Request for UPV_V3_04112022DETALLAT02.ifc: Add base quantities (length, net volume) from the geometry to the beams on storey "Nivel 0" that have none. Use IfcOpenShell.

First a look at what the model holds.

```python
import ifcopenshell
import ifcopenshell.util.element
import ifcopenshell.util.unit

model = ifcopenshell.open("UPV_V3_04112022DETALLAT02.ifc")
print(model.schema)
for unit_type in ("LENGTHUNIT", "AREAUNIT", "VOLUMEUNIT"):
    print(unit_type, ifcopenshell.util.unit.calculate_unit_scale(model, unit_type))
storey = next(s for s in model.by_type("IfcBuildingStorey") if s.Name == "Nivel 0")
beams = [e for e in ifcopenshell.util.element.get_decomposition(storey) if e.is_a("IfcBeam")]
for e in sorted(beams, key=lambda e: e.id()):
    print(e.id(), e.is_a(), e.Name, list(ifcopenshell.util.element.get_psets(e, qtos_only=True)), sep=" | ")
```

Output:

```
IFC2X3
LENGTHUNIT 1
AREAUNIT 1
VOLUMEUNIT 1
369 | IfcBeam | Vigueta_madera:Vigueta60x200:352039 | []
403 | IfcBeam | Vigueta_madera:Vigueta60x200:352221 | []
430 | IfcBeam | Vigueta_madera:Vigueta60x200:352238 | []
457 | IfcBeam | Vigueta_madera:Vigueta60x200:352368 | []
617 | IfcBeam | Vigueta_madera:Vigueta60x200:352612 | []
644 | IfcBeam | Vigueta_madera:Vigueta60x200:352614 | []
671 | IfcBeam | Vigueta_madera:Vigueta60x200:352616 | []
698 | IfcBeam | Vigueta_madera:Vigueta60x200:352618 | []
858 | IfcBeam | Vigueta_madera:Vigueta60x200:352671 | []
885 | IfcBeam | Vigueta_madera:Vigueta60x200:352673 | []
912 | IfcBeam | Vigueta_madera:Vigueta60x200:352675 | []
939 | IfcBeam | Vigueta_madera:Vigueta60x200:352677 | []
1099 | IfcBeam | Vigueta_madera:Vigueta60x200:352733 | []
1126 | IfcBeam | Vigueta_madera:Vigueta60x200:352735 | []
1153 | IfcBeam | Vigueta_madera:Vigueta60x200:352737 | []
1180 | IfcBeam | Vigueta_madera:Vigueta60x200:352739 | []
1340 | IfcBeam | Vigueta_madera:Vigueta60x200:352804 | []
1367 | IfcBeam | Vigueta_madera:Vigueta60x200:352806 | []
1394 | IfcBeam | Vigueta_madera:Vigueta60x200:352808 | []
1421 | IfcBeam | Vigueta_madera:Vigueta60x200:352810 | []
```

```python
import ifcopenshell
import ifcopenshell.api.pset
import ifcopenshell.geom
import ifcopenshell.util.element
import ifcopenshell.util.shape
import ifcopenshell.util.unit

model = ifcopenshell.open("UPV_V3_04112022DETALLAT02.ifc")
unit_scale = ifcopenshell.util.unit.calculate_unit_scale(model)
volume_scale = ifcopenshell.util.unit.calculate_unit_scale(model, "VOLUMEUNIT")
settings = ifcopenshell.geom.settings()

storey = next(s for s in model.by_type("IfcBuildingStorey") if s.Name == "Nivel 0")
beams = [e for e in ifcopenshell.util.element.get_decomposition(storey) if e.is_a("IfcBeam")]

for e in sorted(beams, key=lambda e: e.id()):
    if ifcopenshell.util.element.get_psets(e, qtos_only=True, should_inherit=False):
        continue
    # Geometry comes back in metres, in the element's own axes.
    shape = ifcopenshell.geom.create_shape(settings, e)
    values = {
        "Length": ifcopenshell.util.shape.get_max_xyz(shape.geometry) / unit_scale,
        "NetVolume": ifcopenshell.util.shape.get_volume(shape.geometry) / volume_scale,
    }
    qto = ifcopenshell.api.pset.add_qto(model, product=e, name="BaseQuantities")
    ifcopenshell.api.pset.edit_qto(model, qto=qto, properties=values)
    print(e.id(), {k: round(v, 3) for k, v in values.items()})

model.write("UPV_V3_04112022DETALLAT02_v2.ifc")
```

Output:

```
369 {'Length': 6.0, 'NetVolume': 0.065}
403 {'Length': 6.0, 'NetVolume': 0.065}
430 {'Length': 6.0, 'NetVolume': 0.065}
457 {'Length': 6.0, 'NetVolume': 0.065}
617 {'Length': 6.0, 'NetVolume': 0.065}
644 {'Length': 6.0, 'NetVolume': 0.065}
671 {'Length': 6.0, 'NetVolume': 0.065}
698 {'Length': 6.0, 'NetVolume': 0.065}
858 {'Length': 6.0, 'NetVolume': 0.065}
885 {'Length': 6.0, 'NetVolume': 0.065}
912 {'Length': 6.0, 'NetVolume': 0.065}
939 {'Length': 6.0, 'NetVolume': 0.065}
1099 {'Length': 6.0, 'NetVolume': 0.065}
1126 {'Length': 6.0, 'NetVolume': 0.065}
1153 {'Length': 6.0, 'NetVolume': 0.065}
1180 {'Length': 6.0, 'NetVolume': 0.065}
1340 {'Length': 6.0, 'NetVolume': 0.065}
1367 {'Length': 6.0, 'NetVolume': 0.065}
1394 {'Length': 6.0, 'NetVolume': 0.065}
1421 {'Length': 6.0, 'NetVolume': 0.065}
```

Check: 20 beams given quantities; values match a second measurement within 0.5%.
